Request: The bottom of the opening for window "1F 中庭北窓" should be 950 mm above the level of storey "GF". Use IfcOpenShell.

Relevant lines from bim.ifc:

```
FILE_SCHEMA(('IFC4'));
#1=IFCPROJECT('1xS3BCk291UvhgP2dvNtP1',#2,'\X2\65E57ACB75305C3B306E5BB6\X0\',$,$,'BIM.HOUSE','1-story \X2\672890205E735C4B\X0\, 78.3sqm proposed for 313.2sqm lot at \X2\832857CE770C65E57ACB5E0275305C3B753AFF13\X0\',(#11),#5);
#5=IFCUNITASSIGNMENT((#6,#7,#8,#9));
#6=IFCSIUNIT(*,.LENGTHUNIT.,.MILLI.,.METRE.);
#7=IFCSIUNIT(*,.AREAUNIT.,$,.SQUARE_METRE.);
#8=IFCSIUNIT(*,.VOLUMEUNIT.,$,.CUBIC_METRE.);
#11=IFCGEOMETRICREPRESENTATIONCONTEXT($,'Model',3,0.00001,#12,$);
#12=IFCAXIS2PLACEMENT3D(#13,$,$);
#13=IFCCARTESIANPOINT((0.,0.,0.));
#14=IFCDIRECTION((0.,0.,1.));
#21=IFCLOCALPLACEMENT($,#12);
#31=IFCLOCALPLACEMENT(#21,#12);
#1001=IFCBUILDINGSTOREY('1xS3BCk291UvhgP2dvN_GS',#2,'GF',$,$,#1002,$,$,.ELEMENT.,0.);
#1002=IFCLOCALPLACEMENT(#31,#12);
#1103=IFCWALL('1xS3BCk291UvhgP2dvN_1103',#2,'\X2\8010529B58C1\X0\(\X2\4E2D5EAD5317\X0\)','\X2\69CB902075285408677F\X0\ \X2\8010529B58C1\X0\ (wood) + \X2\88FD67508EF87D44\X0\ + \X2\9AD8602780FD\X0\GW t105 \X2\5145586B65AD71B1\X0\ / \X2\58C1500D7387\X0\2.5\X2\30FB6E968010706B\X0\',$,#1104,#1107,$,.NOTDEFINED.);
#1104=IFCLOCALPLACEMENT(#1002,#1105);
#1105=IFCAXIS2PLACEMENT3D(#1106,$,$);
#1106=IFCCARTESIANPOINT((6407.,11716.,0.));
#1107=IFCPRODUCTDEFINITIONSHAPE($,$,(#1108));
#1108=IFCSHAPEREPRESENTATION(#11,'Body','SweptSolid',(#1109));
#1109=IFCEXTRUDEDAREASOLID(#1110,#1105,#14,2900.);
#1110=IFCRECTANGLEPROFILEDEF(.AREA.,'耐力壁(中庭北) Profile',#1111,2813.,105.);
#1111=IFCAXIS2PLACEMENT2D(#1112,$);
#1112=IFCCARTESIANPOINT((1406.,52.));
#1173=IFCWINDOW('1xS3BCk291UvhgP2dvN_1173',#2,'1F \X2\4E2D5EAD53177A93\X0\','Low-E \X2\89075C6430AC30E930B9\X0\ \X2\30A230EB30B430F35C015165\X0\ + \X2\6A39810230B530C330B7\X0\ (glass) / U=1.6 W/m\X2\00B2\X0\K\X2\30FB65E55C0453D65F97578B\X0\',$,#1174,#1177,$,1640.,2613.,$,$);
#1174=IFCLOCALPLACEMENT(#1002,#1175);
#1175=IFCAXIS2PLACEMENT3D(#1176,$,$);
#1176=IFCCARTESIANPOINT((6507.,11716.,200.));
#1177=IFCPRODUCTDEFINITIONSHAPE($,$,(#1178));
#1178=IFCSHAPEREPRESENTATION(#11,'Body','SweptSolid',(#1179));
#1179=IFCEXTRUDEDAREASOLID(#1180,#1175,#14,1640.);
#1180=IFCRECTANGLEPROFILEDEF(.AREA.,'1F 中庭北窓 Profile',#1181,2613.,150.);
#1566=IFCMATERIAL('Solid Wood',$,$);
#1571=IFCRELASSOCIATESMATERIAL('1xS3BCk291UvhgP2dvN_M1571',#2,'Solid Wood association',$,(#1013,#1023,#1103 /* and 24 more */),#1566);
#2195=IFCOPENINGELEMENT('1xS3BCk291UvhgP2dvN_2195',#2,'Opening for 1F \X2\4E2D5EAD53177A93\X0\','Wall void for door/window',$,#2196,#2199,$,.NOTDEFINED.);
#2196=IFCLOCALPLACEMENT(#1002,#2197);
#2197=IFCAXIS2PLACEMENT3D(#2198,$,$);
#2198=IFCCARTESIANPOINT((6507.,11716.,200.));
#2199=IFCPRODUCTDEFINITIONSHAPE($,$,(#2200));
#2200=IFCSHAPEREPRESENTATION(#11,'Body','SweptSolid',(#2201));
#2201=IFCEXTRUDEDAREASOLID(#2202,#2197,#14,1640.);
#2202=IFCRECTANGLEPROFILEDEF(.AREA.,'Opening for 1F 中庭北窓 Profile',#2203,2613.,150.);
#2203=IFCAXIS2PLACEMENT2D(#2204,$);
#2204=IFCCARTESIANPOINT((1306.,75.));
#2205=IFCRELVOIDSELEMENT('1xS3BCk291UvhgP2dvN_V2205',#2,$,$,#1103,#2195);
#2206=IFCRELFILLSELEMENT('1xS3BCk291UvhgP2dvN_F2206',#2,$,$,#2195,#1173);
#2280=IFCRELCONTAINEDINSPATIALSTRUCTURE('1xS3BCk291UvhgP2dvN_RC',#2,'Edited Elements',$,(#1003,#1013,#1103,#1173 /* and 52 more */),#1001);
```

```python
import numpy as np
import ifcopenshell
import ifcopenshell.api.geometry
import ifcopenshell.geom
import ifcopenshell.util.element
import ifcopenshell.util.placement
import ifcopenshell.util.shape
import ifcopenshell.util.unit

model = ifcopenshell.open("bim.ifc")
unit_scale = ifcopenshell.util.unit.calculate_unit_scale(model)

window = model.by_guid("1xS3BCk291UvhgP2dvN_1173")
opening = window.FillsVoids[0].RelatingOpeningElement
storey = ifcopenshell.util.element.get_container(window, ifc_class="IfcBuildingStorey")
level = ifcopenshell.util.placement.get_local_placement(storey.ObjectPlacement)[2, 3]

# The opening's origin need not be at the sill, so measure its lowest point.
shape = ifcopenshell.geom.create_shape(ifcopenshell.geom.settings(), opening)
bottom = ifcopenshell.util.shape.get_shape_bottom_elevation(shape, shape.geometry) / unit_scale
dz = level + 0.95 / unit_scale - bottom

shift = np.array([0.0, 0.0, dz])
# The window is not placed relative to its opening, so move both.
for product in (opening, window):
    matrix = ifcopenshell.util.placement.get_local_placement(product.ObjectPlacement)
    matrix[:3, 3] += shift
    ifcopenshell.api.geometry.edit_object_placement(model, product=product, matrix=matrix, is_si=False)

print(f"moved by {dz * unit_scale:+.3f} m")

model.write("bim_rev.ifc")
```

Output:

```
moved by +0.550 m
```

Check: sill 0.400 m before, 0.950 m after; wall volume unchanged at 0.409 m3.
